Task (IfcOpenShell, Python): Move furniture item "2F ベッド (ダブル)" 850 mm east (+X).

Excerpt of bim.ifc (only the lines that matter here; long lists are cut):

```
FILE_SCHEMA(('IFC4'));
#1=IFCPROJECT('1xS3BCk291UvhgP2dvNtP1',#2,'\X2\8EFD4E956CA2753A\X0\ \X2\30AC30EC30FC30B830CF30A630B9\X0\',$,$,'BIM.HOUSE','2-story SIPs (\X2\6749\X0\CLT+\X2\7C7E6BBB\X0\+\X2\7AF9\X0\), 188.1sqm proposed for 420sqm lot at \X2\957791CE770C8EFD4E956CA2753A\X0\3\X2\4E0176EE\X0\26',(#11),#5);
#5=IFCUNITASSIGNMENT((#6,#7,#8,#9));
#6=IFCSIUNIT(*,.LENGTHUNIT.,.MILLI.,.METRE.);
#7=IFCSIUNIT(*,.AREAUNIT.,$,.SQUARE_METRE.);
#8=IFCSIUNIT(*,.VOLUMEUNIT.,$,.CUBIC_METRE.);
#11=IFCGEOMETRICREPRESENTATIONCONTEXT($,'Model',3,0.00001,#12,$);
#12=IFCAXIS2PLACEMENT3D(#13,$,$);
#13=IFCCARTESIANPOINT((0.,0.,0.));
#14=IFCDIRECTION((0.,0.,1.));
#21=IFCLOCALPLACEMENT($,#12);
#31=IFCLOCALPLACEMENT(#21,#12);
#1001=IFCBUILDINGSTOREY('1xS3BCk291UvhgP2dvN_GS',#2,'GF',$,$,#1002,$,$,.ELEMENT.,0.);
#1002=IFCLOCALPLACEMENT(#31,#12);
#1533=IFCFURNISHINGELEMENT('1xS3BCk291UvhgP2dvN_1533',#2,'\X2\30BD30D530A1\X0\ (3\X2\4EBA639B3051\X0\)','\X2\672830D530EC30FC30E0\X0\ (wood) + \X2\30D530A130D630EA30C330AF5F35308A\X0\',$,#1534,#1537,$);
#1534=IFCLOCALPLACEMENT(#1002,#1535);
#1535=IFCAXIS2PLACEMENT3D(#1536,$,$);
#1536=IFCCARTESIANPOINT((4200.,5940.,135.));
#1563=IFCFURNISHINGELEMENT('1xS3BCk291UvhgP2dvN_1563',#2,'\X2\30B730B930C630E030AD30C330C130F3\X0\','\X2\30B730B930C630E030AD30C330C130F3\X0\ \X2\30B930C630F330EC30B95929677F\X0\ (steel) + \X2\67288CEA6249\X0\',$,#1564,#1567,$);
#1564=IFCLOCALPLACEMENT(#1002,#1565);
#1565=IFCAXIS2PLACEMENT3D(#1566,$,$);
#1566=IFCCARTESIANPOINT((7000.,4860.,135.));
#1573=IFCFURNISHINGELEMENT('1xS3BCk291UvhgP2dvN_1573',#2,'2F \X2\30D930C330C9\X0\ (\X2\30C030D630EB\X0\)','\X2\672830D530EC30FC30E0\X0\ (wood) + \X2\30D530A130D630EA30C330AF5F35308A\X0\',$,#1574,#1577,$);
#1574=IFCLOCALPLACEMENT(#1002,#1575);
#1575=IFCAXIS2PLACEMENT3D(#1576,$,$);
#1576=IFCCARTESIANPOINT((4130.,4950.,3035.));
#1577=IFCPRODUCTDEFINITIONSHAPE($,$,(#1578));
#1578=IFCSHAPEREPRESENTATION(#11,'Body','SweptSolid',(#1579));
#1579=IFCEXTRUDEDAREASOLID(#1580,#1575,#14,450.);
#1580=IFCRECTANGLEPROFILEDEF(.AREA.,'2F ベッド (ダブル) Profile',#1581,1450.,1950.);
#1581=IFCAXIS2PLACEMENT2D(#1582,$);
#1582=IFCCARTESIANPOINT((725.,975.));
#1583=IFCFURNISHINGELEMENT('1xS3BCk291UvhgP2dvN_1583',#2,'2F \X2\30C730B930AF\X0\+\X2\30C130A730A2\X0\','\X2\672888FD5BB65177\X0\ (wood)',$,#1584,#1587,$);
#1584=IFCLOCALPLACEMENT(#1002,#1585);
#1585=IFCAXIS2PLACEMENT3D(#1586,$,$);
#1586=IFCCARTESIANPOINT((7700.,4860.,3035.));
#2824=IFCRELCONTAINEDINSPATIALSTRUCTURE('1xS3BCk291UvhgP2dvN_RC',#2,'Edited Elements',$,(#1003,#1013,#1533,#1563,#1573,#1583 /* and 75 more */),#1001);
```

```python
import ifcopenshell
import ifcopenshell.api.geometry
import ifcopenshell.util.placement

model = ifcopenshell.open("bim.ifc")

item = model.by_guid("1xS3BCk291UvhgP2dvN_1573")
matrix = ifcopenshell.util.placement.get_local_placement(item.ObjectPlacement)
matrix[0, 3] += 850.0
ifcopenshell.api.geometry.edit_object_placement(model, product=item, matrix=matrix, is_si=False)

print(ifcopenshell.util.placement.get_local_placement(item.ObjectPlacement).round(3) + 0.0)

model.write("bim_rev.ifc")
```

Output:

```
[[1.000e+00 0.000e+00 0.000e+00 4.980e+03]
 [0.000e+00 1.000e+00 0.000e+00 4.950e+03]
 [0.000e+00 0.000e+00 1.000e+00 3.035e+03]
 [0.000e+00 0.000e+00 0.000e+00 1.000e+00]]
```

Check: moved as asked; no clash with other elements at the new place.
